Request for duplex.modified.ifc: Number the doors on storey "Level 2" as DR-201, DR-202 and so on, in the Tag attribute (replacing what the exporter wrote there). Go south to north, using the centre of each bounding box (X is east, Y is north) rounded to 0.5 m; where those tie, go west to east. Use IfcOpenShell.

First a look at what the model holds.

```python
import ifcopenshell
import ifcopenshell.util.element
import ifcopenshell.util.placement

model = ifcopenshell.open("duplex.modified.ifc")
print(model.schema)
storey = next(s for s in model.by_type("IfcBuildingStorey") if s.Name == "Level 2")
doors = [e for e in ifcopenshell.util.element.get_decomposition(storey) if e.is_a("IfcDoor")]
for e in sorted(doors, key=lambda e: e.id()):
    origin = ifcopenshell.util.placement.get_local_placement(e.ObjectPlacement)[:3, 3]
    print(e.id(), e.Tag, e.Name, origin.round(2) + 0.0, sep=" | ")
```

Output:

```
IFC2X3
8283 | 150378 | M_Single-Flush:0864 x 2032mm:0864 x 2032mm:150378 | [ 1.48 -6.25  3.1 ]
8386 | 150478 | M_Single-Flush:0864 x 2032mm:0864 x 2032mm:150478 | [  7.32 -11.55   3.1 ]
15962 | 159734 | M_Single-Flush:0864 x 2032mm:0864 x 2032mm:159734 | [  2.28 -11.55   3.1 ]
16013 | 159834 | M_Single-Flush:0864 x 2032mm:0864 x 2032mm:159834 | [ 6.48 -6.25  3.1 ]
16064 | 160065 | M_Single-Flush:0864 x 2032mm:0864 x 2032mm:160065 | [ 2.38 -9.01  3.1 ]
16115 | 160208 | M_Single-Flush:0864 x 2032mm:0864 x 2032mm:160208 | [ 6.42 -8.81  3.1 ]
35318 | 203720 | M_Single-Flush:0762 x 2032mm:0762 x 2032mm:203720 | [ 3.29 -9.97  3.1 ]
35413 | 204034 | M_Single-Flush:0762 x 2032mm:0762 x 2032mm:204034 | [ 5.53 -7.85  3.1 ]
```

```python
import ifcopenshell
import ifcopenshell.geom
import ifcopenshell.util.element
import ifcopenshell.util.shape

model = ifcopenshell.open("duplex.modified.ifc")
settings = ifcopenshell.geom.settings()
settings.set("use-world-coords", True)


def centre(element):
    shape = ifcopenshell.geom.create_shape(settings, element)
    return ifcopenshell.util.shape.get_bbox_centroid(shape.geometry)


storey = next(s for s in model.by_type("IfcBuildingStorey") if s.Name == "Level 2")
doors = [e for e in ifcopenshell.util.element.get_decomposition(storey) if e.is_a("IfcDoor")]

# Insertion points can sit at a corner or the storey origin, so sort by the geometry (in metres).
centres = {e: centre(e) for e in doors}
doors.sort(key=lambda e: (round(centres[e][1] / 0.5), centres[e][0]))

for i, e in enumerate(doors, start=1):
    number = f"DR-2{i:02d}"
    e.Tag = number
    print(e.id(), number)

model.write("duplex.modified_v2.ifc")
```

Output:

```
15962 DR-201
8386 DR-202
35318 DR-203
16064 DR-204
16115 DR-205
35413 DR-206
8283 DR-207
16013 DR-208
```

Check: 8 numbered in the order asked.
